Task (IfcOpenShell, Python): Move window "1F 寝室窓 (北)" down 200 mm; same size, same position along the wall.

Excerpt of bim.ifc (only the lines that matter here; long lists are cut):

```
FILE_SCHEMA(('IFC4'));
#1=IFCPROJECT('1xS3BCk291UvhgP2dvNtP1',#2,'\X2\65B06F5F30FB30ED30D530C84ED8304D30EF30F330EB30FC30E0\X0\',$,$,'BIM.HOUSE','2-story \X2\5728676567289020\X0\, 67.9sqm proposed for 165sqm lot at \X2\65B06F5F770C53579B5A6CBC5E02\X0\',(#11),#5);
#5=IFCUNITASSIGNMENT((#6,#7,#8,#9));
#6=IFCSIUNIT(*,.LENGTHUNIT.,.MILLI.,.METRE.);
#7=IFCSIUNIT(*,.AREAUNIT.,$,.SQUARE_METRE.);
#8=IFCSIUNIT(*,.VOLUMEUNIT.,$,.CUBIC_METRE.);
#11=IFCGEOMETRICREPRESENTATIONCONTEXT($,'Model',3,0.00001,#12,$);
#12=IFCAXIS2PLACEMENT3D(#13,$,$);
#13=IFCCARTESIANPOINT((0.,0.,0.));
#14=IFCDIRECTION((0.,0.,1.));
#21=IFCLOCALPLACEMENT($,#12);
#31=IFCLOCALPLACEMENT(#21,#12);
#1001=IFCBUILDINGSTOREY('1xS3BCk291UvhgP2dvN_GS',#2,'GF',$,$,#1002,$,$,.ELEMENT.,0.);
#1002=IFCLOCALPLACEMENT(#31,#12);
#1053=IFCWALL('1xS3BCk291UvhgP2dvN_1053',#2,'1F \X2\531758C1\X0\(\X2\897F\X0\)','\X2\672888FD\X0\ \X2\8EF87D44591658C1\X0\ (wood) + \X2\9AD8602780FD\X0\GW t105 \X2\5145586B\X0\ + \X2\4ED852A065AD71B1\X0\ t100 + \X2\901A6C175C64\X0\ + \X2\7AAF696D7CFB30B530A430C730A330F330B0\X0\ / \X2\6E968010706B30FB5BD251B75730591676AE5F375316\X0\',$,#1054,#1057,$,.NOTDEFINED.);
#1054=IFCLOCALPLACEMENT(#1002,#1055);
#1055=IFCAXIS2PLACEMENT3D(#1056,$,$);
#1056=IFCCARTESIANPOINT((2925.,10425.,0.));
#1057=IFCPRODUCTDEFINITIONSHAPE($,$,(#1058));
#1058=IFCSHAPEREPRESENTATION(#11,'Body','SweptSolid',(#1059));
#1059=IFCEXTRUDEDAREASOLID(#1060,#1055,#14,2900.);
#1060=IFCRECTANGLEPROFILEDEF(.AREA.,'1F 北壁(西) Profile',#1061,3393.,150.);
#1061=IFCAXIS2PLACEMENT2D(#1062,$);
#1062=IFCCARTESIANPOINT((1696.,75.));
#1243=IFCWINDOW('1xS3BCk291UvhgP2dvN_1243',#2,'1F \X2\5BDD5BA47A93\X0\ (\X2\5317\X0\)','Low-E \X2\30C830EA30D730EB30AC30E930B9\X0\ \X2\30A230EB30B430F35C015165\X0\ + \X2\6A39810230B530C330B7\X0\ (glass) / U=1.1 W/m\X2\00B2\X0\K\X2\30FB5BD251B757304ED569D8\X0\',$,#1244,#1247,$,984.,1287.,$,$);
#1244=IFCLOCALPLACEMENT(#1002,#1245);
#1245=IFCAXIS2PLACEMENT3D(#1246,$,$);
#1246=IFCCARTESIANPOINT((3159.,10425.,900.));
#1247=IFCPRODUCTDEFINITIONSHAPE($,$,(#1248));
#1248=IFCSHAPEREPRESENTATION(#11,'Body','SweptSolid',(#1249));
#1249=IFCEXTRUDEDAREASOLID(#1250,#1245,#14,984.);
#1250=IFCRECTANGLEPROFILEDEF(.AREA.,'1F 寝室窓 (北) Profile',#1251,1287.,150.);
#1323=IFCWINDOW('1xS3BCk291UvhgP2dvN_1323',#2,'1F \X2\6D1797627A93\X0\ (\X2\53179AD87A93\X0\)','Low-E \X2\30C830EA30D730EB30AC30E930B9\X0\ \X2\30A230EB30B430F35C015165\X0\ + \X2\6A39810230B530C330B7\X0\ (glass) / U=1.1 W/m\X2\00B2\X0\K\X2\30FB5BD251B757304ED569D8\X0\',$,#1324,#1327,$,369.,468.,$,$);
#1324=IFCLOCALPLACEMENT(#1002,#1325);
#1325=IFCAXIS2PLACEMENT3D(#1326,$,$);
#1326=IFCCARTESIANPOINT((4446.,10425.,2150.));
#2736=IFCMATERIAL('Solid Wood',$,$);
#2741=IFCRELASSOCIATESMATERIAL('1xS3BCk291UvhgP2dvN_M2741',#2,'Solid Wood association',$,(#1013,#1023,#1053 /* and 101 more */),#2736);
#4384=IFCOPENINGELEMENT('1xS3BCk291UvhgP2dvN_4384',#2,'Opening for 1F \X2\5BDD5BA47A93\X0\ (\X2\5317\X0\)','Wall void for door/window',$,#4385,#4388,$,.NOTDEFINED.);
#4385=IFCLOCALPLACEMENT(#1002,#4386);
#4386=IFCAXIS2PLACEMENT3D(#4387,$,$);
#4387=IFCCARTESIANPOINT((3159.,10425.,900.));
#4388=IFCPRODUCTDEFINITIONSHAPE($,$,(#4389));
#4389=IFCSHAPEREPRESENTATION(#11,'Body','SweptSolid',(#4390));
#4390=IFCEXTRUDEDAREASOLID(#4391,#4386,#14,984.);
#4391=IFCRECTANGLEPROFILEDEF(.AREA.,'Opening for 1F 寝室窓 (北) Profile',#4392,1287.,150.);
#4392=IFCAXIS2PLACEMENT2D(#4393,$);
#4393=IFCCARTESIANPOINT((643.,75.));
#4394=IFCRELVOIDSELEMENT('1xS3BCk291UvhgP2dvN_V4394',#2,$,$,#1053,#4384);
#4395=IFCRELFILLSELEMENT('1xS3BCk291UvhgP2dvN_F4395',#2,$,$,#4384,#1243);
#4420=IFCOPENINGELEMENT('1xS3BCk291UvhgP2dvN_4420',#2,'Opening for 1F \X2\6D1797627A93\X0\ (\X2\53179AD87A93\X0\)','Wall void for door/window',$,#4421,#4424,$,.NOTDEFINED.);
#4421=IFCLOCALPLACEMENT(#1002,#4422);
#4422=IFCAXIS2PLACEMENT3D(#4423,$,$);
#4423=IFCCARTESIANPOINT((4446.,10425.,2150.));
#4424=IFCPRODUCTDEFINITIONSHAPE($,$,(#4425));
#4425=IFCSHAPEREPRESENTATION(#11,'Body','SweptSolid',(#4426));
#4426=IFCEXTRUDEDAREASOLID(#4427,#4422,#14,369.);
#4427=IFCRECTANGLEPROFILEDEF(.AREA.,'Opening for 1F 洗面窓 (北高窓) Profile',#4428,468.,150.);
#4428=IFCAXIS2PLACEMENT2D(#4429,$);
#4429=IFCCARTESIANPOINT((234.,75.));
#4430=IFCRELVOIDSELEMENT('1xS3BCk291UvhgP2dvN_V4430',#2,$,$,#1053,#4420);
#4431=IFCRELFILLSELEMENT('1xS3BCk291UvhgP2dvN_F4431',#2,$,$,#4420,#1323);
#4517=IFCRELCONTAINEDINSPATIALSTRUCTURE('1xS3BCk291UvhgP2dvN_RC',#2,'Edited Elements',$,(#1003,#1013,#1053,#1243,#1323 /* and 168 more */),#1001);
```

```python
import numpy as np
import ifcopenshell
import ifcopenshell.api.geometry
import ifcopenshell.util.placement
import ifcopenshell.util.unit

model = ifcopenshell.open("bim.ifc")
unit_scale = ifcopenshell.util.unit.calculate_unit_scale(model)

window = model.by_guid("1xS3BCk291UvhgP2dvN_1243")
opening = window.FillsVoids[0].RelatingOpeningElement
dz = -0.2 / unit_scale

shift = np.array([0.0, 0.0, dz])
# The window is not placed relative to its opening, so move both.
for product in (opening, window):
    matrix = ifcopenshell.util.placement.get_local_placement(product.ObjectPlacement)
    matrix[:3, 3] += shift
    ifcopenshell.api.geometry.edit_object_placement(model, product=product, matrix=matrix, is_si=False)

print(f"moved by {dz * unit_scale:+.3f} m")

model.write("bim-out.ifc")
```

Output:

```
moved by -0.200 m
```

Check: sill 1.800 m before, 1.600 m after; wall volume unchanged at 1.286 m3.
